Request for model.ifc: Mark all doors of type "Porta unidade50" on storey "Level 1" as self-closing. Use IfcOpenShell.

First a look at what the model holds.

```python
import ifcopenshell
import ifcopenshell.util.element

model = ifcopenshell.open("model.ifc")
print(model.schema)
storey = next(s for s in model.by_type("IfcBuildingStorey") if s.Name == "Level 1")
doors = [e for e in ifcopenshell.util.element.get_decomposition(storey) if e.is_a("IfcDoor")]
seen = {}
for e in doors:
    element_type = ifcopenshell.util.element.get_type(e)
    key = (element_type.Name if element_type != e and element_type else None, ifcopenshell.util.element.get_pset(e, "Pset_DoorCommon", "SelfClosing"))
    seen[key] = seen.get(key, 0) + 1
for (name, value), count in sorted(seen.items(), key=str):
    print(count, "x", name, "|", value)
```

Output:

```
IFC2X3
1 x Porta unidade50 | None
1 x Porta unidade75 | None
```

```python
import ifcopenshell
import ifcopenshell.api.pset
import ifcopenshell.util.element

model = ifcopenshell.open("model.ifc")

storey = next(s for s in model.by_type("IfcBuildingStorey") if s.Name == "Level 1")
doors = [e for e in ifcopenshell.util.element.get_decomposition(storey) if e.is_a("IfcDoor")]

count = 0
for e in doors:
    element_type = ifcopenshell.util.element.get_type(e)
    if element_type in (None, e) or element_type.Name != "Porta unidade50":
        continue
    # add_pset returns the element's existing set when there is one.
    pset = ifcopenshell.api.pset.add_pset(model, product=e, name="Pset_DoorCommon")
    ifcopenshell.api.pset.edit_pset(model, pset=pset, properties={"SelfClosing": True})
    count += 1

print(count, "doors updated")

model.write("model_edited.ifc")
```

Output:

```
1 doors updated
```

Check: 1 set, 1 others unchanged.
